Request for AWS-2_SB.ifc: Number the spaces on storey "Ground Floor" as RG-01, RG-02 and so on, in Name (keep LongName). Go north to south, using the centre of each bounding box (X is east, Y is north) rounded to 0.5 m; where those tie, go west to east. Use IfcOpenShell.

First a look at what the model holds.

```python
import ifcopenshell
import ifcopenshell.util.element
import ifcopenshell.util.placement

model = ifcopenshell.open("AWS-2_SB.ifc")
print(model.schema)
storey = next(s for s in model.by_type("IfcBuildingStorey") if s.Name == "Ground Floor")
spaces = [e for e in ifcopenshell.util.element.get_decomposition(storey) if e.is_a("IfcSpace")]
for e in sorted(spaces, key=lambda e: e.id()):
    origin = ifcopenshell.util.placement.get_local_placement(e.ObjectPlacement)[:3, 3]
    print(e.id(), e.Name, e.LongName, origin.round(2) + 0.0, sep=" | ")
```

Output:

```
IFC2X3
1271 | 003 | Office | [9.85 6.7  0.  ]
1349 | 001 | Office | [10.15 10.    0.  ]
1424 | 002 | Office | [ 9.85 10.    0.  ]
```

```python
import ifcopenshell
import ifcopenshell.geom
import ifcopenshell.util.element
import ifcopenshell.util.shape

model = ifcopenshell.open("AWS-2_SB.ifc")
settings = ifcopenshell.geom.settings()
settings.set("use-world-coords", True)


def centre(element):
    shape = ifcopenshell.geom.create_shape(settings, element)
    return ifcopenshell.util.shape.get_bbox_centroid(shape.geometry)


storey = next(s for s in model.by_type("IfcBuildingStorey") if s.Name == "Ground Floor")
spaces = [e for e in ifcopenshell.util.element.get_decomposition(storey) if e.is_a("IfcSpace")]

# Insertion points can sit at a corner or the storey origin, so sort by the geometry (in metres).
centres = {e: centre(e) for e in spaces}
spaces.sort(key=lambda e: (-round(centres[e][1] / 0.5), centres[e][0]))

for i, e in enumerate(spaces, start=1):
    number = f"RG-{i:02d}"
    e.Name = number
    print(e.id(), number)

model.write("AWS-2_SB_updated.ifc")
```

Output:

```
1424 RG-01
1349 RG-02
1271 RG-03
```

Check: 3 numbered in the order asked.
